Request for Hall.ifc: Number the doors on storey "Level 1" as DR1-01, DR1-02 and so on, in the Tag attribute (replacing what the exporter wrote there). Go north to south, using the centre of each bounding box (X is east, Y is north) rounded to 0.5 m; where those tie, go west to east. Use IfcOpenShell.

First a look at what the model holds.

```python
import ifcopenshell
import ifcopenshell.util.element
import ifcopenshell.util.placement

model = ifcopenshell.open("Hall.ifc")
print(model.schema)
storey = next(s for s in model.by_type("IfcBuildingStorey") if s.Name == "Level 1")
doors = [e for e in ifcopenshell.util.element.get_decomposition(storey) if e.is_a("IfcDoor")]
for e in sorted(doors, key=lambda e: e.id()):
    origin = ifcopenshell.util.placement.get_local_placement(e.ObjectPlacement)[:3, 3]
    print(e.id(), e.Tag, e.Name, origin.round(2) + 0.0, sep=" | ")
```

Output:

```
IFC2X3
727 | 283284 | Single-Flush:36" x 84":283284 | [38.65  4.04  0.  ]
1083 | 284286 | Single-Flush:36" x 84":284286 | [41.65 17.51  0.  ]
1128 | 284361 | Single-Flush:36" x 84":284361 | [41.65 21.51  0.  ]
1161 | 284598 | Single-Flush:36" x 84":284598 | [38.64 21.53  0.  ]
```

```python
import ifcopenshell
import ifcopenshell.geom
import ifcopenshell.util.element
import ifcopenshell.util.shape

model = ifcopenshell.open("Hall.ifc")
settings = ifcopenshell.geom.settings()
settings.set("use-world-coords", True)


def centre(element):
    shape = ifcopenshell.geom.create_shape(settings, element)
    return ifcopenshell.util.shape.get_bbox_centroid(shape.geometry)


storey = next(s for s in model.by_type("IfcBuildingStorey") if s.Name == "Level 1")
doors = [e for e in ifcopenshell.util.element.get_decomposition(storey) if e.is_a("IfcDoor")]

# Insertion points can sit at a corner or the storey origin, so sort by the geometry (in metres).
centres = {e: centre(e) for e in doors}
doors.sort(key=lambda e: (-round(centres[e][1] / 0.5), centres[e][0]))

for i, e in enumerate(doors, start=1):
    number = f"DR1-{i:02d}"
    e.Tag = number
    print(e.id(), number)

model.write("Hall_updated.ifc")
```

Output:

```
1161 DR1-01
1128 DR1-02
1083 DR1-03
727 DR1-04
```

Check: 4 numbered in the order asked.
